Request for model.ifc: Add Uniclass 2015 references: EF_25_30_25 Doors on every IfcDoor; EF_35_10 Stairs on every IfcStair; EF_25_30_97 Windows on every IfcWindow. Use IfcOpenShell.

First a look at what the model holds.

```python
import ifcopenshell

model = ifcopenshell.open("model.ifc")
print(model.schema)
print("classifications:", [c.Name for c in model.by_type("IfcClassification")])
for ifc_class in ("IfcDoor", "IfcRoof", "IfcStair", "IfcWall", "IfcWindow"):
    print(ifc_class, len(model.by_type(ifc_class)))
```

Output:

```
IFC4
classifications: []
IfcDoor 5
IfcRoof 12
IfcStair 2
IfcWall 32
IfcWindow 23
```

```python
import ifcopenshell
import ifcopenshell.api.classification

model = ifcopenshell.open("model.ifc")

system = ifcopenshell.api.classification.add_classification(model, classification="Uniclass 2015")

codes = {
    "IfcDoor": ("EF_25_30_25", "Doors"),
    "IfcStair": ("EF_35_10", "Stairs"),
    "IfcWindow": ("EF_25_30_97", "Windows"),
}
for ifc_class, (code, name) in codes.items():
    products = model.by_type(ifc_class)
    ifcopenshell.api.classification.add_reference(
        model, products=products, classification=system, identification=code, name=name
    )
    print(code, len(products))

model.write("model_v2.ifc")
```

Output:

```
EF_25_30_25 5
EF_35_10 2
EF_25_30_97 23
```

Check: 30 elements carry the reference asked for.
